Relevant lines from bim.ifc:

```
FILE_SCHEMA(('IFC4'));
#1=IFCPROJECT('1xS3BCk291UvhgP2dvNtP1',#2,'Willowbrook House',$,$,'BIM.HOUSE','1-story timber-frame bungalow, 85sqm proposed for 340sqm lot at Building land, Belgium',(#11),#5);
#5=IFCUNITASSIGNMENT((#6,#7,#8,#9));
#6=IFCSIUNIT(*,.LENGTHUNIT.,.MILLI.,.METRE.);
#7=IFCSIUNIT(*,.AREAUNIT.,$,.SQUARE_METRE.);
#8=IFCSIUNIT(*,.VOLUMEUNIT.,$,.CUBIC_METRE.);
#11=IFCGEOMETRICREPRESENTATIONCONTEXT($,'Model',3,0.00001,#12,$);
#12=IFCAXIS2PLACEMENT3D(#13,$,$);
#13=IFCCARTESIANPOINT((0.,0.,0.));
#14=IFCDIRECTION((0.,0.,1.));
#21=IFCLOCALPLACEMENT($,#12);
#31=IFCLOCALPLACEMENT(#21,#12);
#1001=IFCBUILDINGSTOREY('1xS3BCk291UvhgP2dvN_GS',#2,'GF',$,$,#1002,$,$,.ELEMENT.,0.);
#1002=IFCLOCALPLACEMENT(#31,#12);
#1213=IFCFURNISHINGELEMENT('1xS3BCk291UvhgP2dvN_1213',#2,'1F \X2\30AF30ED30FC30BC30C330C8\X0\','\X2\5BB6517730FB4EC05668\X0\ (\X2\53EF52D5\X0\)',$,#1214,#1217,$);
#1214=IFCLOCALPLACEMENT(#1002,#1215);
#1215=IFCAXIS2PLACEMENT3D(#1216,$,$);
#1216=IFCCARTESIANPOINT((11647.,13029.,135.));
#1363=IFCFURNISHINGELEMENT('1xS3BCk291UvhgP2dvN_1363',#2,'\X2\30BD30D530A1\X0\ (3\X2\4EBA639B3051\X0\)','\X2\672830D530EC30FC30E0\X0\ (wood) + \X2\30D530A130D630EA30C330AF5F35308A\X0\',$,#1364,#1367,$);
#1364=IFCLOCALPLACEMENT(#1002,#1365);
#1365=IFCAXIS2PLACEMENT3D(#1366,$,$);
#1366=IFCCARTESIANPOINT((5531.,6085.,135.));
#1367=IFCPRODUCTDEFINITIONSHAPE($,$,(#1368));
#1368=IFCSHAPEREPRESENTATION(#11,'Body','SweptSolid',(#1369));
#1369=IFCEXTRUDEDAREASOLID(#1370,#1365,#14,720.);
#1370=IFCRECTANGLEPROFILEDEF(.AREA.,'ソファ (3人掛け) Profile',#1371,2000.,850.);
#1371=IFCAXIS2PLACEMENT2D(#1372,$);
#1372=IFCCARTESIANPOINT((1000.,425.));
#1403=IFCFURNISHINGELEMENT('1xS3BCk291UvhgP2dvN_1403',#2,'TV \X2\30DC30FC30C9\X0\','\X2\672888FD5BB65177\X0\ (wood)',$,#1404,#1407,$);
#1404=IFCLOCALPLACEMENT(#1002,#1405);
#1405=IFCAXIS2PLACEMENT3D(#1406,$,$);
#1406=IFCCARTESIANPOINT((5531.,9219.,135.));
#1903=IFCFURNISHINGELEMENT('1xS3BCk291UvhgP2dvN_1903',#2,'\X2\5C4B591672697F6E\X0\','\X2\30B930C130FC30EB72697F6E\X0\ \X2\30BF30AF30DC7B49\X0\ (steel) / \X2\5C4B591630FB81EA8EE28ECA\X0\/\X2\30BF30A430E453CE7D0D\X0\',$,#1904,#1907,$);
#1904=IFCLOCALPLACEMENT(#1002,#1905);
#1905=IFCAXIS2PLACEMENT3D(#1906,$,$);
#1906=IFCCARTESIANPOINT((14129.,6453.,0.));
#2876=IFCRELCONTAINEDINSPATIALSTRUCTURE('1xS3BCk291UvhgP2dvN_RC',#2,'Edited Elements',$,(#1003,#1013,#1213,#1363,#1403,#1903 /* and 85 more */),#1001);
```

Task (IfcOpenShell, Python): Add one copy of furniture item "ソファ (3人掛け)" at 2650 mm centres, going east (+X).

```python
import numpy as np
import ifcopenshell
import ifcopenshell.api.geometry
import ifcopenshell.api.root
import ifcopenshell.util.element
import ifcopenshell.util.placement
import ifcopenshell.util.unit

model = ifcopenshell.open("bim.ifc")
unit_scale = ifcopenshell.util.unit.calculate_unit_scale(model)


def reuse_history(source, copy):
    """copy_class also copies each property set's owner history, people and application; keep the originals."""
    for rel in copy.IsDefinedBy:
        if rel.is_a("IfcRelDefinesByProperties") and (history := rel.RelatingPropertyDefinition.OwnerHistory):
            rel.RelatingPropertyDefinition.OwnerHistory = source.OwnerHistory
            ifcopenshell.util.element.remove_deep2(model, history)


source = model.by_id(1363)
base = ifcopenshell.util.placement.get_local_placement(source.ObjectPlacement)
step = np.array([1.0, 0.0, 0.0]) * 2.65 / unit_scale

for i in range(1, 2):
    copy = ifcopenshell.api.root.copy_class(model, product=source)
    copy.Representation = ifcopenshell.util.element.copy_deep(
        model, source.Representation, exclude=["IfcGeometricRepresentationContext", "IfcRepresentationMap"]
    )
    reuse_history(source, copy)
    matrix = base.copy()
    matrix[:3, 3] += i * step
    print("added at", matrix[:3, 3].round(3) + 0.0)
    ifcopenshell.api.geometry.edit_object_placement(model, product=copy, matrix=matrix, is_si=False)

model.write("bim_rev.ifc")
```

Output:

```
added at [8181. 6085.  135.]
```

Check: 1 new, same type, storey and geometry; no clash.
